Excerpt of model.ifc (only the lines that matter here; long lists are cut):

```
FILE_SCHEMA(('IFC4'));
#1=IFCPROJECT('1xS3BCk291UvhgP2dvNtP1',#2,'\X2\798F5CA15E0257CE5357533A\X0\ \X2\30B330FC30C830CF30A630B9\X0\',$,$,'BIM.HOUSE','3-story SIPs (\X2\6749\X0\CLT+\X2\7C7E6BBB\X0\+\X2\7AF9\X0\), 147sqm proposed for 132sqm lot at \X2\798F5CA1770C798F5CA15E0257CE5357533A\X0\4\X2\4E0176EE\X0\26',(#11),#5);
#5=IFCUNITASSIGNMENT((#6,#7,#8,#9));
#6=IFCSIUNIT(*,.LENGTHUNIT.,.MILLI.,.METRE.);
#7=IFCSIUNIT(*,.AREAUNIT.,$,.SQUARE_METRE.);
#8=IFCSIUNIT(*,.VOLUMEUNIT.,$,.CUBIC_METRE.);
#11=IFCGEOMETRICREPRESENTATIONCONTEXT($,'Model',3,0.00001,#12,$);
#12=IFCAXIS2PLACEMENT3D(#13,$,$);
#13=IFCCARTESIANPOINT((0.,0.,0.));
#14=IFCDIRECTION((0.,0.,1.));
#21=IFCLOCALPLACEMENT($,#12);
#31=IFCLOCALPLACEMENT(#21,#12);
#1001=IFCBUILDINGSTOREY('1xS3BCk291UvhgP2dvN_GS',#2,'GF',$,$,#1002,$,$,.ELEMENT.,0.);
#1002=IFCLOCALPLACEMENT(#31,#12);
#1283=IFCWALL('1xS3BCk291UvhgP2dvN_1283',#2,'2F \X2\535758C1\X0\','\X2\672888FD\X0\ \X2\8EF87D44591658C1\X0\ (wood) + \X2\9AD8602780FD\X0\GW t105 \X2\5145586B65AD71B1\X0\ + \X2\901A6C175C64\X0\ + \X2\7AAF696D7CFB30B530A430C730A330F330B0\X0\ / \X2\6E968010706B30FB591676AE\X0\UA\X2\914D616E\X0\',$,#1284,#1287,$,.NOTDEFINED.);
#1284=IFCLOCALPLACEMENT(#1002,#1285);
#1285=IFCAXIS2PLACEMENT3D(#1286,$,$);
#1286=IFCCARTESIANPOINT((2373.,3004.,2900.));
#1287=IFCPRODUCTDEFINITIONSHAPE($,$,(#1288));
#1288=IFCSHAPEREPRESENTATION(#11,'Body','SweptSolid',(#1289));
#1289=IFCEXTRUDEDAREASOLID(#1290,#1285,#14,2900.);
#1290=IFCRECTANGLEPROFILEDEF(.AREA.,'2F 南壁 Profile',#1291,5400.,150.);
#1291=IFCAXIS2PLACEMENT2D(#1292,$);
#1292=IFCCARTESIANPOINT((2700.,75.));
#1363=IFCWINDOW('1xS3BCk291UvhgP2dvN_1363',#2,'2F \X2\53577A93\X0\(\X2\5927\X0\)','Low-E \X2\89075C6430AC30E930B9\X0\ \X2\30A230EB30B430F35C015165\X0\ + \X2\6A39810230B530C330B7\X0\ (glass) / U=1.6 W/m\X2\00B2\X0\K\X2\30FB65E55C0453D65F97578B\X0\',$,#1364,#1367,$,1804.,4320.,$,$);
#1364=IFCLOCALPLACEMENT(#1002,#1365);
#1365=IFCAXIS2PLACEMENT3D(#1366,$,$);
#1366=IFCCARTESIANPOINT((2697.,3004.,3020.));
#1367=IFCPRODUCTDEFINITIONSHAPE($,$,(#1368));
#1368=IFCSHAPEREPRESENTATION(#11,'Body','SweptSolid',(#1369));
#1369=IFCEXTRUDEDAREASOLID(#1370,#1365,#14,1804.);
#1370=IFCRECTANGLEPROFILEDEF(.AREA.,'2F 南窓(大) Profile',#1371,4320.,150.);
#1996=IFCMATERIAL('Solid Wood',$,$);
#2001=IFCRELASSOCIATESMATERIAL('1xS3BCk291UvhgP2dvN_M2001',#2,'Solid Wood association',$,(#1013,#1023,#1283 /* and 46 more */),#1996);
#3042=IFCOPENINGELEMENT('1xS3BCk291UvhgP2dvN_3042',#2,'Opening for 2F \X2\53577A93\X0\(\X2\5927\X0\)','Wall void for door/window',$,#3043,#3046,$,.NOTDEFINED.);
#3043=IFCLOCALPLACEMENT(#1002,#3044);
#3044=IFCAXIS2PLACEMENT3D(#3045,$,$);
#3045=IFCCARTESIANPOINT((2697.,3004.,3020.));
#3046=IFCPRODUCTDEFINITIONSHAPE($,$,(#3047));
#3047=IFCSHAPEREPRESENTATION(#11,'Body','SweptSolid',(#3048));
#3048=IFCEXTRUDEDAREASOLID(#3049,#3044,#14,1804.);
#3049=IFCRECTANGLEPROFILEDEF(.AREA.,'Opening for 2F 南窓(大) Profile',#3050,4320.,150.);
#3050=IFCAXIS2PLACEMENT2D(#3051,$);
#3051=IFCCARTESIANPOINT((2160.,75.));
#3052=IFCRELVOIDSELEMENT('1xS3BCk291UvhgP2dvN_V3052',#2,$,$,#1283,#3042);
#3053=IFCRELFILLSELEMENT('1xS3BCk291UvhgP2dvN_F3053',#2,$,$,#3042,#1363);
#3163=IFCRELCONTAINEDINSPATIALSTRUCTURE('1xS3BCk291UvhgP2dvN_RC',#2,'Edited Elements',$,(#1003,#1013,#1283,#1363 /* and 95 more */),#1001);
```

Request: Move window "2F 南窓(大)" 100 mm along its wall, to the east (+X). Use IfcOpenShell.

```python
import ifcopenshell
import ifcopenshell.api.geometry
import ifcopenshell.util.placement
import ifcopenshell.util.unit

model = ifcopenshell.open("model.ifc")
unit_scale = ifcopenshell.util.unit.calculate_unit_scale(model)

window = model.by_id(1363)
opening = window.FillsVoids[0].RelatingOpeningElement
wall = opening.VoidsElements[0].RelatingBuildingElement

wall_matrix = ifcopenshell.util.placement.get_local_placement(wall.ObjectPlacement)
shift = wall_matrix[:3, 0] * 0.1 / unit_scale
before = ifcopenshell.util.placement.get_local_placement(window.ObjectPlacement)[:3, 3].copy()

# The window is not placed relative to its opening, so move both.
for product in (opening, window):
    matrix = ifcopenshell.util.placement.get_local_placement(product.ObjectPlacement)
    matrix[:3, 3] += shift
    ifcopenshell.api.geometry.edit_object_placement(model, product=product, matrix=matrix, is_si=False)

after = ifcopenshell.util.placement.get_local_placement(window.ObjectPlacement)[:3, 3]
print("window moved by", (after - before).round(3) + 0.0)

model.write("model_updated.ifc")
```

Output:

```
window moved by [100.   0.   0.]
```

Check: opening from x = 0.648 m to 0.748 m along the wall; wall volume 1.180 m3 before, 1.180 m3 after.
